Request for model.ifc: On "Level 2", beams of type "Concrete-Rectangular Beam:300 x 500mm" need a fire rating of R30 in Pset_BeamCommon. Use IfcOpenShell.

First a look at what the model holds.

```python
import ifcopenshell
import ifcopenshell.util.element

model = ifcopenshell.open("model.ifc")
print(model.schema)
storey = next(s for s in model.by_type("IfcBuildingStorey") if s.Name == "Level 2")
beams = [e for e in ifcopenshell.util.element.get_decomposition(storey) if e.is_a("IfcBeam")]
seen = {}
for e in beams:
    element_type = ifcopenshell.util.element.get_type(e)
    key = (element_type.Name if element_type != e and element_type else None, ifcopenshell.util.element.get_pset(e, "Pset_BeamCommon", "FireRating"))
    seen[key] = seen.get(key, 0) + 1
for (name, value), count in sorted(seen.items(), key=str):
    print(count, "x", name, "|", value)
```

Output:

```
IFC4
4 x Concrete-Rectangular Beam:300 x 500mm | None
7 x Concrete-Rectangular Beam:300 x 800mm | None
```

```python
import ifcopenshell
import ifcopenshell.api.pset
import ifcopenshell.util.element

model = ifcopenshell.open("model.ifc")

storey = next(s for s in model.by_type("IfcBuildingStorey") if s.Name == "Level 2")
beams = [e for e in ifcopenshell.util.element.get_decomposition(storey) if e.is_a("IfcBeam")]

count = 0
for e in beams:
    element_type = ifcopenshell.util.element.get_type(e)
    if element_type in (None, e) or element_type.Name != "Concrete-Rectangular Beam:300 x 500mm":
        continue
    # add_pset returns the element's existing set when there is one.
    pset = ifcopenshell.api.pset.add_pset(model, product=e, name="Pset_BeamCommon")
    ifcopenshell.api.pset.edit_pset(model, pset=pset, properties={"FireRating": "R30"})
    count += 1

print(count, "beams updated")

model.write("model_v2.ifc")
```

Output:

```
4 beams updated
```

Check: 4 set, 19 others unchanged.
